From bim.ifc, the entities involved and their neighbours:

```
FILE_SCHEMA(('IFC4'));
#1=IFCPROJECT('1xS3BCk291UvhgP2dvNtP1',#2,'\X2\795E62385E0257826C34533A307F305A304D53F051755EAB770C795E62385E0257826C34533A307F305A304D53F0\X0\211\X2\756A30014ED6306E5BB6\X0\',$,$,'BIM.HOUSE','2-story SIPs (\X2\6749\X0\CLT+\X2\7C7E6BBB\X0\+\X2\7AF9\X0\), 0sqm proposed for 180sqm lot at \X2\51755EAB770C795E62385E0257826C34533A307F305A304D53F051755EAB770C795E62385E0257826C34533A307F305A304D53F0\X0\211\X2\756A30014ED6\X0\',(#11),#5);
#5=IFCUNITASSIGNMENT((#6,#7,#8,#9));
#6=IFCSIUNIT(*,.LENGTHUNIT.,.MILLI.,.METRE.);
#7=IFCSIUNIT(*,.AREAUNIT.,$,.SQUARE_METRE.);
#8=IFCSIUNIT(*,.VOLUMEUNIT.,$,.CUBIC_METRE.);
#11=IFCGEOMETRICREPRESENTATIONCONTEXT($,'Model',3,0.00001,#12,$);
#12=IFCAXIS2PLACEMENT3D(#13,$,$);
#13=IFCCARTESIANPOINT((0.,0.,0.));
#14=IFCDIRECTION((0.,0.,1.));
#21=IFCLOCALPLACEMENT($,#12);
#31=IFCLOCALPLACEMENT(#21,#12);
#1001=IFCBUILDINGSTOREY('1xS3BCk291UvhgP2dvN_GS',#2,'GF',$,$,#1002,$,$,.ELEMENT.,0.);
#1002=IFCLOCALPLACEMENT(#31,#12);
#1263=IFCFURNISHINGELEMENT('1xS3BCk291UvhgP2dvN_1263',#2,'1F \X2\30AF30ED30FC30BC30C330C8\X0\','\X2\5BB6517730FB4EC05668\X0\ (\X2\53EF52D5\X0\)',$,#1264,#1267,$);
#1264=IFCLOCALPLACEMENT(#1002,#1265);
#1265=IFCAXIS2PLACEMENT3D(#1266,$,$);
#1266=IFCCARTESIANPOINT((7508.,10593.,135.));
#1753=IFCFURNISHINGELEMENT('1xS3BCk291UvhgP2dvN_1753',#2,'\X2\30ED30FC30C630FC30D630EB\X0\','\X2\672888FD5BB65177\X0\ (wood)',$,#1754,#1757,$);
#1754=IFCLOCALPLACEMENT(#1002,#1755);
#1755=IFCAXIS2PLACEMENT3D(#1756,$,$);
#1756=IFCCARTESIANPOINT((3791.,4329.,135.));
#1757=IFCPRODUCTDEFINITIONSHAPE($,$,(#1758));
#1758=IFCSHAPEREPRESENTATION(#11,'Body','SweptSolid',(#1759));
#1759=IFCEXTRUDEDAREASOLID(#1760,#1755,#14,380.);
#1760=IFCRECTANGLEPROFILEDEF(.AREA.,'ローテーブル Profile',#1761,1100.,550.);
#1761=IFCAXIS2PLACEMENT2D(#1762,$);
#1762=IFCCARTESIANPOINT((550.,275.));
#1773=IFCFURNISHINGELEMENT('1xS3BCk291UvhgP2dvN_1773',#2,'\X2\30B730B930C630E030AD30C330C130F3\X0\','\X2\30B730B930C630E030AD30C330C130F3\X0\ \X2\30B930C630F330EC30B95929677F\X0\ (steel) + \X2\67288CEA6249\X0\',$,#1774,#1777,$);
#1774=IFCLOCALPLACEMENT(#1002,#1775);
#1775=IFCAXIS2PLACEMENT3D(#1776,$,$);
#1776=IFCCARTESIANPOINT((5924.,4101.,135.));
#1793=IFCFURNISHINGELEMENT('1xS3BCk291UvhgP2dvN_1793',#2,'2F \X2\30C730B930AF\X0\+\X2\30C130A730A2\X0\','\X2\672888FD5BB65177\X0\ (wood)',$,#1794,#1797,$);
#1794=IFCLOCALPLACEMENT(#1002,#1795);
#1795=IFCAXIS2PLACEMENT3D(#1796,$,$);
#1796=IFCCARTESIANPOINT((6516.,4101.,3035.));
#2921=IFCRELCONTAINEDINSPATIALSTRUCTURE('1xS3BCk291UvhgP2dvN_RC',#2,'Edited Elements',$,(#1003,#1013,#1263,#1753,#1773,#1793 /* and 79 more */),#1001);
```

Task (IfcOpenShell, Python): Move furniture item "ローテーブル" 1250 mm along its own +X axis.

```python
import ifcopenshell
import ifcopenshell.api.geometry
import ifcopenshell.util.placement
import ifcopenshell.util.unit

model = ifcopenshell.open("bim.ifc")
unit_scale = ifcopenshell.util.unit.calculate_unit_scale(model)

item = model.by_guid("1xS3BCk291UvhgP2dvN_1753")
matrix = ifcopenshell.util.placement.get_local_placement(item.ObjectPlacement)
matrix[:3, 3] += matrix[:3, 0] * 1.25 / unit_scale
ifcopenshell.api.geometry.edit_object_placement(model, product=item, matrix=matrix, is_si=False)

print(ifcopenshell.util.placement.get_local_placement(item.ObjectPlacement).round(3) + 0.0)

model.write("bim_v2.ifc")
```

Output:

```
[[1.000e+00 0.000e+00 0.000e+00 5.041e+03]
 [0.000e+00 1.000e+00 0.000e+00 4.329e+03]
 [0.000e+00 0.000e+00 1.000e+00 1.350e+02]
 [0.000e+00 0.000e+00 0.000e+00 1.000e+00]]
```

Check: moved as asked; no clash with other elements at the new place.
